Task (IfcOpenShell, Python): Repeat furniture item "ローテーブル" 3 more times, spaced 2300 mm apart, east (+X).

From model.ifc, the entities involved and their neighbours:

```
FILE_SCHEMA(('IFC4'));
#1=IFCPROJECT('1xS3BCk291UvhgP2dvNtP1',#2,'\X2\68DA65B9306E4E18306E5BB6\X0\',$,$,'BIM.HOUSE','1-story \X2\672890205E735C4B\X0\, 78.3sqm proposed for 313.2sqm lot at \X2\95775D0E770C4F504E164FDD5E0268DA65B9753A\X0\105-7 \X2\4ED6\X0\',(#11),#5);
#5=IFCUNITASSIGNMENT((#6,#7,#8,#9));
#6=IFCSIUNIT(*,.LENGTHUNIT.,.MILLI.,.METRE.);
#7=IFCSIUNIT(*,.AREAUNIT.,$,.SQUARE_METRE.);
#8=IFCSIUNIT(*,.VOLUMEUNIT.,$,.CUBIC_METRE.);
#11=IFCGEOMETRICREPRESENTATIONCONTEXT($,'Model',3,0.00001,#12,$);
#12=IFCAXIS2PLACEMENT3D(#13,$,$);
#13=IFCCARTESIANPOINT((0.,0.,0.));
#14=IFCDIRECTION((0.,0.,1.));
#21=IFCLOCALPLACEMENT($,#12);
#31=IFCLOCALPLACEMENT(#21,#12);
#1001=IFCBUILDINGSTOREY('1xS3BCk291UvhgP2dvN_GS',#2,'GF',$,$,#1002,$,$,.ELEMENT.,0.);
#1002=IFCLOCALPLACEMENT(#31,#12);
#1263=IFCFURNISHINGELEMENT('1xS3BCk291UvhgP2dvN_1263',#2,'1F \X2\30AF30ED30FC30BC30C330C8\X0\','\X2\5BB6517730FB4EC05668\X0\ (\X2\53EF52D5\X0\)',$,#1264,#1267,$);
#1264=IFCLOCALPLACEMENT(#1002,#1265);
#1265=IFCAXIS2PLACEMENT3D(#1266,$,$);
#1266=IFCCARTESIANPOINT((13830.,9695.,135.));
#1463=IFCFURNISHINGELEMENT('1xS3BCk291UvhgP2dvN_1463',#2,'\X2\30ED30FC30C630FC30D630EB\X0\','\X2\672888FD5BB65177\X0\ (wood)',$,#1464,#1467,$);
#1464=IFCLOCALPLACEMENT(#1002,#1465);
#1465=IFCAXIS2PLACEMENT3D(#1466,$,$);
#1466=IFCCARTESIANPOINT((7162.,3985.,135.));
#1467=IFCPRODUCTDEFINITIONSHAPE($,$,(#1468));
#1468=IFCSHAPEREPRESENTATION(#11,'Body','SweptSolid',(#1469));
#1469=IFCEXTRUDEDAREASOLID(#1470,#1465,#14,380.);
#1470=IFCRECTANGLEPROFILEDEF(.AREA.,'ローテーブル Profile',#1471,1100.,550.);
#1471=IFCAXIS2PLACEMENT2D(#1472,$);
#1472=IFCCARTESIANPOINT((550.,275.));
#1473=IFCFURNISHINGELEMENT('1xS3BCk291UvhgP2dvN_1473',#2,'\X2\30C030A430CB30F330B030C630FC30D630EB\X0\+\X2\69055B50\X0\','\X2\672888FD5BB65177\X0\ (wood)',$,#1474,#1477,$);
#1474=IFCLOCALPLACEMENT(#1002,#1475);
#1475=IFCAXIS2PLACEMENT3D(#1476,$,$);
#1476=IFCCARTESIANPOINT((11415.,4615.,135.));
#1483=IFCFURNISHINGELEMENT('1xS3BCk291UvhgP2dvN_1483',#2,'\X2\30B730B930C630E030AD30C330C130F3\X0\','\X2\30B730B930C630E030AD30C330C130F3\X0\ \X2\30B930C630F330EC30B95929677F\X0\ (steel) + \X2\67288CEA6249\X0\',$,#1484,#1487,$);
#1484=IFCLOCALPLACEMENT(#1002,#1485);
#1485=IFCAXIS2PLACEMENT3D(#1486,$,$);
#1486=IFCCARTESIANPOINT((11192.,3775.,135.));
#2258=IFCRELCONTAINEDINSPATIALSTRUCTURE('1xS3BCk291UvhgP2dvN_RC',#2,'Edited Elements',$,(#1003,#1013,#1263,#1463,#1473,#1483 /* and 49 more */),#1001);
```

```python
import numpy as np
import ifcopenshell
import ifcopenshell.api.geometry
import ifcopenshell.api.root
import ifcopenshell.util.element
import ifcopenshell.util.placement
import ifcopenshell.util.unit

model = ifcopenshell.open("model.ifc")
unit_scale = ifcopenshell.util.unit.calculate_unit_scale(model)


def reuse_history(source, copy):
    """copy_class also copies each property set's owner history, people and application; keep the originals."""
    for rel in copy.IsDefinedBy:
        if rel.is_a("IfcRelDefinesByProperties") and (history := rel.RelatingPropertyDefinition.OwnerHistory):
            rel.RelatingPropertyDefinition.OwnerHistory = source.OwnerHistory
            ifcopenshell.util.element.remove_deep2(model, history)


source = model.by_guid("1xS3BCk291UvhgP2dvN_1463")
base = ifcopenshell.util.placement.get_local_placement(source.ObjectPlacement)
step = np.array([1.0, 0.0, 0.0]) * 2.3 / unit_scale

for i in range(1, 4):
    copy = ifcopenshell.api.root.copy_class(model, product=source)
    copy.Representation = ifcopenshell.util.element.copy_deep(
        model, source.Representation, exclude=["IfcGeometricRepresentationContext", "IfcRepresentationMap"]
    )
    reuse_history(source, copy)
    matrix = base.copy()
    matrix[:3, 3] += i * step
    print("added at", matrix[:3, 3].round(3) + 0.0)
    ifcopenshell.api.geometry.edit_object_placement(model, product=copy, matrix=matrix, is_si=False)

model.write("model_v2.ifc")
```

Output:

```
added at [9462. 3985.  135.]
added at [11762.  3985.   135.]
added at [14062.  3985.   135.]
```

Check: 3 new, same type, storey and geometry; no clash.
